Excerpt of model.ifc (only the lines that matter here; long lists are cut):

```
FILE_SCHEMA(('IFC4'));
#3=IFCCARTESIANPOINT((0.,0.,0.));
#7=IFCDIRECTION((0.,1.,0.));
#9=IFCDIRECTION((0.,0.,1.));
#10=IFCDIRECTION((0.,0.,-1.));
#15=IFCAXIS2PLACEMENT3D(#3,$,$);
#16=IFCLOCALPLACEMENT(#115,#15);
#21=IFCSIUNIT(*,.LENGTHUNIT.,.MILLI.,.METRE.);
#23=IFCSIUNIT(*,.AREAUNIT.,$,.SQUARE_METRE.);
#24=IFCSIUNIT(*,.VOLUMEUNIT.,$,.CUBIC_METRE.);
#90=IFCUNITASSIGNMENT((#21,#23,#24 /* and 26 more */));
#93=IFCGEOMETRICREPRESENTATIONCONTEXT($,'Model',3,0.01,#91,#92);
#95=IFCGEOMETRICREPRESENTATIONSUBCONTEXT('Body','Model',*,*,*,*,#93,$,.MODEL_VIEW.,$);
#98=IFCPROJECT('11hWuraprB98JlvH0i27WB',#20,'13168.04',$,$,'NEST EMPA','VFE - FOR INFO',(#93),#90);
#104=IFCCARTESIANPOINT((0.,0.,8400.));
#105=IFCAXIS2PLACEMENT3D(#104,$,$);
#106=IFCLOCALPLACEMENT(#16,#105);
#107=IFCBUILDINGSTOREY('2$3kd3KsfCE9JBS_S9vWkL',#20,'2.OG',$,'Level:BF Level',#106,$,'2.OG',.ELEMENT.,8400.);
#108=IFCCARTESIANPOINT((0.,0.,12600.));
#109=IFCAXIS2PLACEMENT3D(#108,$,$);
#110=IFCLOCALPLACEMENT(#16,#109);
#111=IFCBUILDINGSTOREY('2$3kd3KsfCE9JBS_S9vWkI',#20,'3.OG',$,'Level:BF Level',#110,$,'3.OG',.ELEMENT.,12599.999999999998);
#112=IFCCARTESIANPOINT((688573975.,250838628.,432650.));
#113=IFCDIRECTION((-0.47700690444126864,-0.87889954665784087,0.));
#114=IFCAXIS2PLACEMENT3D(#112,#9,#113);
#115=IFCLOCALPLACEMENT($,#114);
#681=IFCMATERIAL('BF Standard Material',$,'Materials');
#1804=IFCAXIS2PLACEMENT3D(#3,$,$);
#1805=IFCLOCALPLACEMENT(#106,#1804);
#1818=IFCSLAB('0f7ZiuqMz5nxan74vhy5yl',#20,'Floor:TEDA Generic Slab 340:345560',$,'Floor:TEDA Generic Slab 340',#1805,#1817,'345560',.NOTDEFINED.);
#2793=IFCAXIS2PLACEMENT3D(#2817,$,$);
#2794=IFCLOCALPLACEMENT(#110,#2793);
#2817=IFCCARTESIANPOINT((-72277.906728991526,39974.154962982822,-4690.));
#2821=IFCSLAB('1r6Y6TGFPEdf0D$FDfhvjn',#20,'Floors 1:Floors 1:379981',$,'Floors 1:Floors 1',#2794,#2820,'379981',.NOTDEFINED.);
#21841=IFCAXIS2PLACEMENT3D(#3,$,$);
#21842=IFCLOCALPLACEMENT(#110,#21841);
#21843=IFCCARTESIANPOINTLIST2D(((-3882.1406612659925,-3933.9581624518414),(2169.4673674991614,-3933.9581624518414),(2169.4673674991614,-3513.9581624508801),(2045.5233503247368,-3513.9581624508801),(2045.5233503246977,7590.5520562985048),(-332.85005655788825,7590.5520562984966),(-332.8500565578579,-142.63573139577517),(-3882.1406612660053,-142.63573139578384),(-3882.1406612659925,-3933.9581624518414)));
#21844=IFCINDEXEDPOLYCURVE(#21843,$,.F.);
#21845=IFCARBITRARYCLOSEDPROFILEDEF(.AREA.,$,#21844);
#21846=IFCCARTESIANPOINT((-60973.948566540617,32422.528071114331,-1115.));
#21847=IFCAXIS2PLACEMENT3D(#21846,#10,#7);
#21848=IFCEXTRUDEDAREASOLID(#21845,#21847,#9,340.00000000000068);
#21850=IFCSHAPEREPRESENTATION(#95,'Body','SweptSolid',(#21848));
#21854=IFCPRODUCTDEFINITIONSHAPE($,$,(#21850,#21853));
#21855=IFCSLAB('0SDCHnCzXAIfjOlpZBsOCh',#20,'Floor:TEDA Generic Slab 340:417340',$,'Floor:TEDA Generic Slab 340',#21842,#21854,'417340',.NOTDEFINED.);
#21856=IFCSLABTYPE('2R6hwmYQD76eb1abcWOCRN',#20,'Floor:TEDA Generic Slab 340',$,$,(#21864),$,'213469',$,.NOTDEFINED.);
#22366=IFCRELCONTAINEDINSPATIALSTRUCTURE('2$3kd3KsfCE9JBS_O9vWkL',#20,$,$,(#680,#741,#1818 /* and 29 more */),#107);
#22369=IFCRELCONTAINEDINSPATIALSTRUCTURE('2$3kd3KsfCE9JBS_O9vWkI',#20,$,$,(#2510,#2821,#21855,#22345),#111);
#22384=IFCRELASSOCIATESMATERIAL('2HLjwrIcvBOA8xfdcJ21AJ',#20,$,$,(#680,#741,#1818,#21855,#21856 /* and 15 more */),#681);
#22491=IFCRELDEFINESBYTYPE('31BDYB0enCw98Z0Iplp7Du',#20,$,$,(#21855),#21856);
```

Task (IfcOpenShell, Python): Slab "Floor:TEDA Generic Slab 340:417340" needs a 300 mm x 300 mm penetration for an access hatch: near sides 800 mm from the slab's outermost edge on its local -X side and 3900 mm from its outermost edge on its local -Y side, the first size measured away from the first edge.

```python
import numpy as np
import ifcopenshell
import ifcopenshell.api.feature
import ifcopenshell.api.geometry
import ifcopenshell.api.root
import ifcopenshell.geom
import ifcopenshell.util.placement
import ifcopenshell.util.representation
import ifcopenshell.util.shape
import ifcopenshell.util.unit

model = ifcopenshell.open("model.ifc")
unit_scale = ifcopenshell.util.unit.calculate_unit_scale(model)
settings = ifcopenshell.geom.settings()


def volume(element):
    """Net volume in cubic metres, openings subtracted."""
    shape = ifcopenshell.geom.create_shape(settings, element)
    return ifcopenshell.util.shape.get_volume(shape.geometry)


slab = model.by_id(21855)
before = volume(slab)

# Extent in the slab's own axes, in metres. The edges named are its -X and -Y sides.
slab_shape = ifcopenshell.geom.create_shape(settings, slab)
vertices = ifcopenshell.util.shape.get_vertices(slab_shape.geometry)
x_min, y_min, bottom = vertices.min(axis=0)
top = vertices[:, 2].max()

opening = ifcopenshell.api.root.create_entity(model, ifc_class="IfcOpeningElement", name="Access hatch opening", predefined_type="OPENING")
context = ifcopenshell.util.representation.get_context(model, "Model", "Body", "MODEL_VIEW")
width, depth = 0.3, 0.3
outline = [(0.0, 0.0), (width, 0.0), (width, depth), (0.0, depth), (0.0, 0.0)]
# Overshoot both faces by 50 mm so the cut is clean.
shape = ifcopenshell.api.geometry.add_slab_representation(
    model, context=context, depth=top - bottom + 0.1, polyline=outline
)
ifcopenshell.api.geometry.assign_representation(model, product=opening, representation=shape)

matrix = ifcopenshell.util.placement.get_local_placement(slab.ObjectPlacement)
matrix[:, 3] = matrix @ np.append(np.array([x_min + 0.8, y_min + 3.9, bottom - 0.05]) / unit_scale, 1.0)
ifcopenshell.api.geometry.edit_object_placement(model, product=opening, matrix=matrix, is_si=False)
ifcopenshell.api.feature.add_feature(model, feature=opening, element=slab)

after = volume(slab)

print(f"slab volume {before:.3f} -> {after:.3f} m3")

model.write("model_edited.ifc")
```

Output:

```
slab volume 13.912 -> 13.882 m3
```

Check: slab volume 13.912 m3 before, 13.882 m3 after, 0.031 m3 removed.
